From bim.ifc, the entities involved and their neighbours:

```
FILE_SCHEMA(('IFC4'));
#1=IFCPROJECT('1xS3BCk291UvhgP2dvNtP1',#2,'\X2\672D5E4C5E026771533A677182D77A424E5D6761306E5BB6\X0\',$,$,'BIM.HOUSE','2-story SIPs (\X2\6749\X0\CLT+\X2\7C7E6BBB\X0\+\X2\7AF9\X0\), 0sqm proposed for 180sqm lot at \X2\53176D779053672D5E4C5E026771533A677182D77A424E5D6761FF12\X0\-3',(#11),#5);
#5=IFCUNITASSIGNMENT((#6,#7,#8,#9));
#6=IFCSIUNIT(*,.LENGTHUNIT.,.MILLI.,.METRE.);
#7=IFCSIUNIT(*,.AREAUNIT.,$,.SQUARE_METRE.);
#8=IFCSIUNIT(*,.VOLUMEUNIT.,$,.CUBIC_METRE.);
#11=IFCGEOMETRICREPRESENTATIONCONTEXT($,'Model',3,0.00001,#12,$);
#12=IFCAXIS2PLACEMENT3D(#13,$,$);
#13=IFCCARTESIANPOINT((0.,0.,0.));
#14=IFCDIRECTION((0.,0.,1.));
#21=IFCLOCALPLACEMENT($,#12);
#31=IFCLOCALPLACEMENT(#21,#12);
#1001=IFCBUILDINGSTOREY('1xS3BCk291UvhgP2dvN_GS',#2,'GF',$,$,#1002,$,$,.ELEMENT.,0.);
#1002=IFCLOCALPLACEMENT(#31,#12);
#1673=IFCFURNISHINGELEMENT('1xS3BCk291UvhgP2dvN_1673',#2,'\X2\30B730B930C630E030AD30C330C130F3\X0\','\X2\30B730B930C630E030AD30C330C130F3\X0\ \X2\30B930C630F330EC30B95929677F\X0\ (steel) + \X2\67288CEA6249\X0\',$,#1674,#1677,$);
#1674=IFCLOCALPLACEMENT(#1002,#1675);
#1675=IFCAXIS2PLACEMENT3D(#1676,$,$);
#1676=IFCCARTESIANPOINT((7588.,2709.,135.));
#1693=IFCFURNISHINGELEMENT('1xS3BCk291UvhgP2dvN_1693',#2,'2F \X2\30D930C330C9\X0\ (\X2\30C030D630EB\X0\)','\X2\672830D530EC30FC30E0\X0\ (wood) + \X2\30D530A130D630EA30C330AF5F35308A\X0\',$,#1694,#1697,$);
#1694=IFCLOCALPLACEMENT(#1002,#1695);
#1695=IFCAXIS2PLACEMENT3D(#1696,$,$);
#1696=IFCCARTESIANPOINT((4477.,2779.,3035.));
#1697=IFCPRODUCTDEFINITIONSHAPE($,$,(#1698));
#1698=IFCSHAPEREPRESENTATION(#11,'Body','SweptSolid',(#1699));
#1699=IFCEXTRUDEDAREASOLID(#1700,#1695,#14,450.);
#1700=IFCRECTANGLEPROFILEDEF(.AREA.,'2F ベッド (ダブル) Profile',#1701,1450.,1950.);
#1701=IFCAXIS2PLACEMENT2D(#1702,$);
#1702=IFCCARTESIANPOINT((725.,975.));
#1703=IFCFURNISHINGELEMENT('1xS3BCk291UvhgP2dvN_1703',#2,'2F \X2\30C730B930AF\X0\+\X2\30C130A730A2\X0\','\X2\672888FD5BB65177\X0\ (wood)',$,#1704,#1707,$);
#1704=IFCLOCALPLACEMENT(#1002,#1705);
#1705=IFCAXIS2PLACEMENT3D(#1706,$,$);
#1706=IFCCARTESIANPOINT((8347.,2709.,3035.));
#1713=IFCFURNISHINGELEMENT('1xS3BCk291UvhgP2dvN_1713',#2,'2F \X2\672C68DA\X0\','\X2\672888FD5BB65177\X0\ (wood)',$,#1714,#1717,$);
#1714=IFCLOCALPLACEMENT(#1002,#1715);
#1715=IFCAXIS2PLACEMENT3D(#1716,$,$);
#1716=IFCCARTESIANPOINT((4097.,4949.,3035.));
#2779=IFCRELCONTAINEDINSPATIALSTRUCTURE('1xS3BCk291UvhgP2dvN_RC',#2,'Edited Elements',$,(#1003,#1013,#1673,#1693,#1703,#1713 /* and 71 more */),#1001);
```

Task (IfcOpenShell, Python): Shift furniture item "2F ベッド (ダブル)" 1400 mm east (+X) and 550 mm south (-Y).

```python
import ifcopenshell
import ifcopenshell.api.geometry
import ifcopenshell.util.placement

model = ifcopenshell.open("bim.ifc")

item = model.by_guid("1xS3BCk291UvhgP2dvN_1693")
matrix = ifcopenshell.util.placement.get_local_placement(item.ObjectPlacement)
matrix[0, 3] += 1400.0
matrix[1, 3] -= 550.0
ifcopenshell.api.geometry.edit_object_placement(model, product=item, matrix=matrix, is_si=False)

print(ifcopenshell.util.placement.get_local_placement(item.ObjectPlacement).round(3) + 0.0)

model.write("bim_edited.ifc")
```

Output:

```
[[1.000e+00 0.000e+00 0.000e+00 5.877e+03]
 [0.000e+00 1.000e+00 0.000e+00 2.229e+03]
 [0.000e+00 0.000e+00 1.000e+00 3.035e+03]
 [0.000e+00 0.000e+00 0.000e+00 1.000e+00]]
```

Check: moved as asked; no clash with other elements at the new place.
